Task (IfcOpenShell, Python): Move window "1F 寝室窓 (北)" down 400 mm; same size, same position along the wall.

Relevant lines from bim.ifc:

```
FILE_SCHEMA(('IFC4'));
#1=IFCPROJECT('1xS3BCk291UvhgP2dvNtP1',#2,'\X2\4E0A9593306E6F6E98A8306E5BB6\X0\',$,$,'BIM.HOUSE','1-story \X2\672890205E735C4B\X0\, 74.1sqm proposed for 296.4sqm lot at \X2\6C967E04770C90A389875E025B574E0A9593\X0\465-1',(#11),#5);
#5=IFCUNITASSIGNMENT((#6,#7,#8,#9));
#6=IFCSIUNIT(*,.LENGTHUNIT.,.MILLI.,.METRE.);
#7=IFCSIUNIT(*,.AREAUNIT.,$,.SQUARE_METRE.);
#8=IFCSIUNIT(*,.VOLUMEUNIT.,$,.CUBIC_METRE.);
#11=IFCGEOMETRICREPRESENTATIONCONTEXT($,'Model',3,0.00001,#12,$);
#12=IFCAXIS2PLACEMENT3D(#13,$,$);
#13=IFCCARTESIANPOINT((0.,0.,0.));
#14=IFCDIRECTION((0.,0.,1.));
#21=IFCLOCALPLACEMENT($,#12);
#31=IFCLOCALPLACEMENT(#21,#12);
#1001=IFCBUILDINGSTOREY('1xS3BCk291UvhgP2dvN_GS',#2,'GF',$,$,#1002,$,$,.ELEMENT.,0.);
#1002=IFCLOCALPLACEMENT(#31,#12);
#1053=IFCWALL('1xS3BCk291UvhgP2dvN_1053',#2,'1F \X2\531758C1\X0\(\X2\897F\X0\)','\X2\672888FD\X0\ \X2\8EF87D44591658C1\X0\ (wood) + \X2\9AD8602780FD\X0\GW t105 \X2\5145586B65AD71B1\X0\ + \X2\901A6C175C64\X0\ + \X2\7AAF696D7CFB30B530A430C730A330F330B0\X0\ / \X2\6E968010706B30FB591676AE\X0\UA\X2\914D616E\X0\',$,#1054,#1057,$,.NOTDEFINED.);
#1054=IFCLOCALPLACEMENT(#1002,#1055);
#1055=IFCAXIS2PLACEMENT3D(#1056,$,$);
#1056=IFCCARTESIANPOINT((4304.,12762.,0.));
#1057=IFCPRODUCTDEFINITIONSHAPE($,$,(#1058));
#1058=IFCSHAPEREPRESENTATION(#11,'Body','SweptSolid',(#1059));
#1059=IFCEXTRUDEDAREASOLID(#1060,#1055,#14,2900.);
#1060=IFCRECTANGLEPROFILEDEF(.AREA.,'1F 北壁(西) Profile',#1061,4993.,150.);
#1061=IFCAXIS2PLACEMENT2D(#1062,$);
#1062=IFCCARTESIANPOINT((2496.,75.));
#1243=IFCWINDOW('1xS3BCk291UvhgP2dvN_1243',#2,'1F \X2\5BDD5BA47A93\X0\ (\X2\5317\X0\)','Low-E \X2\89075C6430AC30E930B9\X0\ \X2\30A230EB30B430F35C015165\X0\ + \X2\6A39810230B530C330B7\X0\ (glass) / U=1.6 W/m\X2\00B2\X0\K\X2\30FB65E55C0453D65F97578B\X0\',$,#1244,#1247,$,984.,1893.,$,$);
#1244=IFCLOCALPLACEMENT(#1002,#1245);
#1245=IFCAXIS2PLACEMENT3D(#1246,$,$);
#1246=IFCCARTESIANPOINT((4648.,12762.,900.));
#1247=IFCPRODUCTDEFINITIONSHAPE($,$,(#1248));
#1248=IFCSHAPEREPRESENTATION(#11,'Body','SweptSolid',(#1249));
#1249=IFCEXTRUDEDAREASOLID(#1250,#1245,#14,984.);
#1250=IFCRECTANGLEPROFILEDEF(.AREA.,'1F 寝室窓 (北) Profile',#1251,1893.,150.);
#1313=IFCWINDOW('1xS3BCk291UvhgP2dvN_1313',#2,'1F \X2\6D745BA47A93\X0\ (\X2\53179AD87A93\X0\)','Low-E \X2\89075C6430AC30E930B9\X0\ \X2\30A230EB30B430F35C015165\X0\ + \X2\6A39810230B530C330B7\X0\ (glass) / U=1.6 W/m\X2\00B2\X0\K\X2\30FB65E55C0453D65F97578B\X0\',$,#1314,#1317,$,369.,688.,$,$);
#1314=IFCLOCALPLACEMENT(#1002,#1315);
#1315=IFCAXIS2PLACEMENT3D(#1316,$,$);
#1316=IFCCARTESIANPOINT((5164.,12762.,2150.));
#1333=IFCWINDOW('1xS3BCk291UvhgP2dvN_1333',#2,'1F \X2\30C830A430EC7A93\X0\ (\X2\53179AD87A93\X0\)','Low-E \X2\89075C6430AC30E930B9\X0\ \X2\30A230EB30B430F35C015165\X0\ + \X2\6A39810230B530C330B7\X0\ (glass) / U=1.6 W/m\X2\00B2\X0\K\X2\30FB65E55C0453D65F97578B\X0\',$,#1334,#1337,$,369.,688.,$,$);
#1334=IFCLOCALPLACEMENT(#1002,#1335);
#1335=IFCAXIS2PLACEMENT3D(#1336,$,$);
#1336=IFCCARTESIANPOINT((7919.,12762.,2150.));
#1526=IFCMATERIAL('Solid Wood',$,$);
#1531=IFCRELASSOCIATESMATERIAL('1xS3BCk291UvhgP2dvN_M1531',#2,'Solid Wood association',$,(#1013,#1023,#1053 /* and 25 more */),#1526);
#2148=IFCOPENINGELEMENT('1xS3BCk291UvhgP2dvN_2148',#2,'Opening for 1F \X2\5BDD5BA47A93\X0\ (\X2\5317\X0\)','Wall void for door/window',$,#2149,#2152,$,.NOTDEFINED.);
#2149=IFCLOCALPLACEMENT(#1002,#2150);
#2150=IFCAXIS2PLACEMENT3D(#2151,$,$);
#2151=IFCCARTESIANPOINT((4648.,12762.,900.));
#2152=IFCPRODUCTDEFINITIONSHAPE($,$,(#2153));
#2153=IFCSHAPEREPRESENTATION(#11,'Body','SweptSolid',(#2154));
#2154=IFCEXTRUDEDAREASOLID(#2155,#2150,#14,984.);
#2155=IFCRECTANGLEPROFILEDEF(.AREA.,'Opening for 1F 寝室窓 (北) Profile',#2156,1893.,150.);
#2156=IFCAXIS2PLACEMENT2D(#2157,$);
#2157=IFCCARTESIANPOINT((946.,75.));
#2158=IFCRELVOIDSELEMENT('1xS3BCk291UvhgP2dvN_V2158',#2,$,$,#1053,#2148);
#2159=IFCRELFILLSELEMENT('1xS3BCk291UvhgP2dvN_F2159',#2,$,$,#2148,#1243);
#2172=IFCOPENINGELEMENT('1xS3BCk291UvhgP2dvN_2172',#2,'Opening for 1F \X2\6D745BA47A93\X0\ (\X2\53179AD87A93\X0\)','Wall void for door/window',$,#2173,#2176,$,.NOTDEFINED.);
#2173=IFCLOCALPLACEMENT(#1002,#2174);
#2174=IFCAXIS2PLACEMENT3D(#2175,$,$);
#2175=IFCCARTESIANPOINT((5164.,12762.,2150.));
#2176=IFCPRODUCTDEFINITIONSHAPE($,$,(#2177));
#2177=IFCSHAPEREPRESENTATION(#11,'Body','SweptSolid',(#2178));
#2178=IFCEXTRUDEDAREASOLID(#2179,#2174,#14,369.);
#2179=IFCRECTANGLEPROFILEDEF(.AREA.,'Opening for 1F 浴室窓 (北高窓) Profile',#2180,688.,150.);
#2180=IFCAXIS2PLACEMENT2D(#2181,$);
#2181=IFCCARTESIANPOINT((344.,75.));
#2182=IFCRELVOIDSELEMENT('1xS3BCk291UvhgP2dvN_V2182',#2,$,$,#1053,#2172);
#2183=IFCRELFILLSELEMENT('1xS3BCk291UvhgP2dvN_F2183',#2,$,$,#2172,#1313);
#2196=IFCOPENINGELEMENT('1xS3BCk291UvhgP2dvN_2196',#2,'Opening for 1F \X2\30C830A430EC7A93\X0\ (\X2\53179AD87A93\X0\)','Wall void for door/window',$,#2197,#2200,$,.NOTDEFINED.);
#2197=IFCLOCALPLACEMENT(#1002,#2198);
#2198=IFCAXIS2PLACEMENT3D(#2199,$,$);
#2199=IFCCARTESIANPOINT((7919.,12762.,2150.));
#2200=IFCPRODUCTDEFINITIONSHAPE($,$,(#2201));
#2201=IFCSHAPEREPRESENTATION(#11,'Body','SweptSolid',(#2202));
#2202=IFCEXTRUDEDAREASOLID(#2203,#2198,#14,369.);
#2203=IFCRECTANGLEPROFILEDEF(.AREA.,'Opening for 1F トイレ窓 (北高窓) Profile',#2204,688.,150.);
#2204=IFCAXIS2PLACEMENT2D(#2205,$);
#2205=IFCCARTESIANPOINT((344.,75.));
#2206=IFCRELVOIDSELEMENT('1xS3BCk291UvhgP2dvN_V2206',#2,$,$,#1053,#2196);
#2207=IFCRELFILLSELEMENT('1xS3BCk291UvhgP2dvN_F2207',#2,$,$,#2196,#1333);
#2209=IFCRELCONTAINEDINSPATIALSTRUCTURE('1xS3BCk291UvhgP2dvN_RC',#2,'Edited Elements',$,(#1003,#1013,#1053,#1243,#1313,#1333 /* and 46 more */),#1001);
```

```python
import numpy as np
import ifcopenshell
import ifcopenshell.api.geometry
import ifcopenshell.util.placement
import ifcopenshell.util.unit

model = ifcopenshell.open("bim.ifc")
unit_scale = ifcopenshell.util.unit.calculate_unit_scale(model)

window = model.by_guid("1xS3BCk291UvhgP2dvN_1243")
opening = window.FillsVoids[0].RelatingOpeningElement
dz = -400.0

shift = np.array([0.0, 0.0, dz])
# The window is not placed relative to its opening, so move both.
for product in (opening, window):
    matrix = ifcopenshell.util.placement.get_local_placement(product.ObjectPlacement)
    matrix[:3, 3] += shift
    ifcopenshell.api.geometry.edit_object_placement(model, product=product, matrix=matrix, is_si=False)

print(f"moved by {dz * unit_scale:+.3f} m")

model.write("bim-out.ifc")
```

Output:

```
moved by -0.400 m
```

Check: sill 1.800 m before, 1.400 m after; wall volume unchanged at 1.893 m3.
